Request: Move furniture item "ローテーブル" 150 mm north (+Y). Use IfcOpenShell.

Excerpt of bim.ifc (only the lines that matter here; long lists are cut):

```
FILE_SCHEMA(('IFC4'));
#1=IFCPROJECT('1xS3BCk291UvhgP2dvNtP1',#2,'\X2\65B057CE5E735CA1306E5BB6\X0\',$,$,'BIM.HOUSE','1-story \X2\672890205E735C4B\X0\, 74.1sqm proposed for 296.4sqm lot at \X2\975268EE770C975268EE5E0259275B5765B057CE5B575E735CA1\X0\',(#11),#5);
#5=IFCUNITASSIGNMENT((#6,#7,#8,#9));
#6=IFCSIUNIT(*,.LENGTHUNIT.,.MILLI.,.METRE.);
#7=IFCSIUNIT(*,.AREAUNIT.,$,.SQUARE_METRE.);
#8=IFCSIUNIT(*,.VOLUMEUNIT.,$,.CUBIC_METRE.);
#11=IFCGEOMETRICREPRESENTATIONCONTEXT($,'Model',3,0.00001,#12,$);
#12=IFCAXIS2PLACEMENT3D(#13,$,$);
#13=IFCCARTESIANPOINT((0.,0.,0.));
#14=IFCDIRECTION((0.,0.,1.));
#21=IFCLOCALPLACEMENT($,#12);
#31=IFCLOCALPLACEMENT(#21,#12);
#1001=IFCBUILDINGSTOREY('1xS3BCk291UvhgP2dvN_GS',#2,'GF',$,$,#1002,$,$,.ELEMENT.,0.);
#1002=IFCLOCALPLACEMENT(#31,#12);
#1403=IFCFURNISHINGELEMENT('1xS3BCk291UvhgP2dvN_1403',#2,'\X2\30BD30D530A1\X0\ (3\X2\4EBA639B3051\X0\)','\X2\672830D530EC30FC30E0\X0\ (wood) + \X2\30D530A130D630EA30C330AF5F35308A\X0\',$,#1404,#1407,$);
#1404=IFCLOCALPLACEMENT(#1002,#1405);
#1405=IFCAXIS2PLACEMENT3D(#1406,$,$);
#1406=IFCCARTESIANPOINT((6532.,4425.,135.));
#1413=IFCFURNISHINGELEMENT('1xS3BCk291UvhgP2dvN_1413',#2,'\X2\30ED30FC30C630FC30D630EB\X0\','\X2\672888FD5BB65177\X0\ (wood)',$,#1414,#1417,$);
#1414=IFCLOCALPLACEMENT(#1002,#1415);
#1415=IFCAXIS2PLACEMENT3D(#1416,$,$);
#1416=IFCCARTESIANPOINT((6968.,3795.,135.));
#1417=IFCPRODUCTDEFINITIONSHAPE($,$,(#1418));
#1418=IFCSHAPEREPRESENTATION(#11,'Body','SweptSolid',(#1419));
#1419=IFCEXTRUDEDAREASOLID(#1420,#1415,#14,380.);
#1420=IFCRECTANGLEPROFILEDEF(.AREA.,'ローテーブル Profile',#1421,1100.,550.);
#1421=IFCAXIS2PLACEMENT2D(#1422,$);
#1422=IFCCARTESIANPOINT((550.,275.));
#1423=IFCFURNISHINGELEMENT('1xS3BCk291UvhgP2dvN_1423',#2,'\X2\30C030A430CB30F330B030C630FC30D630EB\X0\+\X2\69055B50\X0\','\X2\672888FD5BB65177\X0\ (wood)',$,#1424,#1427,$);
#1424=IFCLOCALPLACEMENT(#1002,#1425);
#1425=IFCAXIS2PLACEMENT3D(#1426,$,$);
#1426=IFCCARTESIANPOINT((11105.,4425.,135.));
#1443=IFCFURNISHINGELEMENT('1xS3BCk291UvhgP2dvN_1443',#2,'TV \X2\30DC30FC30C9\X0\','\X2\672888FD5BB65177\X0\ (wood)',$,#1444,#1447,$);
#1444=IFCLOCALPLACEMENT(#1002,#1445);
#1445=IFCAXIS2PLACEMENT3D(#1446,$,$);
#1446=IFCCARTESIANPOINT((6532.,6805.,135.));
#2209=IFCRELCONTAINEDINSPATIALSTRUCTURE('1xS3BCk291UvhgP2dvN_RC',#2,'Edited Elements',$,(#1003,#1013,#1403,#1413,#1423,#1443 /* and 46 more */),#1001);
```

```python
import ifcopenshell
import ifcopenshell.api.geometry
import ifcopenshell.util.placement
import ifcopenshell.util.unit

model = ifcopenshell.open("bim.ifc")
unit_scale = ifcopenshell.util.unit.calculate_unit_scale(model)

item = model.by_guid("1xS3BCk291UvhgP2dvN_1413")
matrix = ifcopenshell.util.placement.get_local_placement(item.ObjectPlacement)
matrix[1, 3] += 0.15 / unit_scale
ifcopenshell.api.geometry.edit_object_placement(model, product=item, matrix=matrix, is_si=False)

print(ifcopenshell.util.placement.get_local_placement(item.ObjectPlacement).round(3) + 0.0)

model.write("bim_rev.ifc")
```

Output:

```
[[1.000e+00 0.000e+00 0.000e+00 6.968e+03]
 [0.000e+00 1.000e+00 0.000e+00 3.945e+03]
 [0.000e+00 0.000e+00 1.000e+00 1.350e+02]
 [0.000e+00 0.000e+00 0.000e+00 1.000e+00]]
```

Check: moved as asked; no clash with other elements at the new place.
